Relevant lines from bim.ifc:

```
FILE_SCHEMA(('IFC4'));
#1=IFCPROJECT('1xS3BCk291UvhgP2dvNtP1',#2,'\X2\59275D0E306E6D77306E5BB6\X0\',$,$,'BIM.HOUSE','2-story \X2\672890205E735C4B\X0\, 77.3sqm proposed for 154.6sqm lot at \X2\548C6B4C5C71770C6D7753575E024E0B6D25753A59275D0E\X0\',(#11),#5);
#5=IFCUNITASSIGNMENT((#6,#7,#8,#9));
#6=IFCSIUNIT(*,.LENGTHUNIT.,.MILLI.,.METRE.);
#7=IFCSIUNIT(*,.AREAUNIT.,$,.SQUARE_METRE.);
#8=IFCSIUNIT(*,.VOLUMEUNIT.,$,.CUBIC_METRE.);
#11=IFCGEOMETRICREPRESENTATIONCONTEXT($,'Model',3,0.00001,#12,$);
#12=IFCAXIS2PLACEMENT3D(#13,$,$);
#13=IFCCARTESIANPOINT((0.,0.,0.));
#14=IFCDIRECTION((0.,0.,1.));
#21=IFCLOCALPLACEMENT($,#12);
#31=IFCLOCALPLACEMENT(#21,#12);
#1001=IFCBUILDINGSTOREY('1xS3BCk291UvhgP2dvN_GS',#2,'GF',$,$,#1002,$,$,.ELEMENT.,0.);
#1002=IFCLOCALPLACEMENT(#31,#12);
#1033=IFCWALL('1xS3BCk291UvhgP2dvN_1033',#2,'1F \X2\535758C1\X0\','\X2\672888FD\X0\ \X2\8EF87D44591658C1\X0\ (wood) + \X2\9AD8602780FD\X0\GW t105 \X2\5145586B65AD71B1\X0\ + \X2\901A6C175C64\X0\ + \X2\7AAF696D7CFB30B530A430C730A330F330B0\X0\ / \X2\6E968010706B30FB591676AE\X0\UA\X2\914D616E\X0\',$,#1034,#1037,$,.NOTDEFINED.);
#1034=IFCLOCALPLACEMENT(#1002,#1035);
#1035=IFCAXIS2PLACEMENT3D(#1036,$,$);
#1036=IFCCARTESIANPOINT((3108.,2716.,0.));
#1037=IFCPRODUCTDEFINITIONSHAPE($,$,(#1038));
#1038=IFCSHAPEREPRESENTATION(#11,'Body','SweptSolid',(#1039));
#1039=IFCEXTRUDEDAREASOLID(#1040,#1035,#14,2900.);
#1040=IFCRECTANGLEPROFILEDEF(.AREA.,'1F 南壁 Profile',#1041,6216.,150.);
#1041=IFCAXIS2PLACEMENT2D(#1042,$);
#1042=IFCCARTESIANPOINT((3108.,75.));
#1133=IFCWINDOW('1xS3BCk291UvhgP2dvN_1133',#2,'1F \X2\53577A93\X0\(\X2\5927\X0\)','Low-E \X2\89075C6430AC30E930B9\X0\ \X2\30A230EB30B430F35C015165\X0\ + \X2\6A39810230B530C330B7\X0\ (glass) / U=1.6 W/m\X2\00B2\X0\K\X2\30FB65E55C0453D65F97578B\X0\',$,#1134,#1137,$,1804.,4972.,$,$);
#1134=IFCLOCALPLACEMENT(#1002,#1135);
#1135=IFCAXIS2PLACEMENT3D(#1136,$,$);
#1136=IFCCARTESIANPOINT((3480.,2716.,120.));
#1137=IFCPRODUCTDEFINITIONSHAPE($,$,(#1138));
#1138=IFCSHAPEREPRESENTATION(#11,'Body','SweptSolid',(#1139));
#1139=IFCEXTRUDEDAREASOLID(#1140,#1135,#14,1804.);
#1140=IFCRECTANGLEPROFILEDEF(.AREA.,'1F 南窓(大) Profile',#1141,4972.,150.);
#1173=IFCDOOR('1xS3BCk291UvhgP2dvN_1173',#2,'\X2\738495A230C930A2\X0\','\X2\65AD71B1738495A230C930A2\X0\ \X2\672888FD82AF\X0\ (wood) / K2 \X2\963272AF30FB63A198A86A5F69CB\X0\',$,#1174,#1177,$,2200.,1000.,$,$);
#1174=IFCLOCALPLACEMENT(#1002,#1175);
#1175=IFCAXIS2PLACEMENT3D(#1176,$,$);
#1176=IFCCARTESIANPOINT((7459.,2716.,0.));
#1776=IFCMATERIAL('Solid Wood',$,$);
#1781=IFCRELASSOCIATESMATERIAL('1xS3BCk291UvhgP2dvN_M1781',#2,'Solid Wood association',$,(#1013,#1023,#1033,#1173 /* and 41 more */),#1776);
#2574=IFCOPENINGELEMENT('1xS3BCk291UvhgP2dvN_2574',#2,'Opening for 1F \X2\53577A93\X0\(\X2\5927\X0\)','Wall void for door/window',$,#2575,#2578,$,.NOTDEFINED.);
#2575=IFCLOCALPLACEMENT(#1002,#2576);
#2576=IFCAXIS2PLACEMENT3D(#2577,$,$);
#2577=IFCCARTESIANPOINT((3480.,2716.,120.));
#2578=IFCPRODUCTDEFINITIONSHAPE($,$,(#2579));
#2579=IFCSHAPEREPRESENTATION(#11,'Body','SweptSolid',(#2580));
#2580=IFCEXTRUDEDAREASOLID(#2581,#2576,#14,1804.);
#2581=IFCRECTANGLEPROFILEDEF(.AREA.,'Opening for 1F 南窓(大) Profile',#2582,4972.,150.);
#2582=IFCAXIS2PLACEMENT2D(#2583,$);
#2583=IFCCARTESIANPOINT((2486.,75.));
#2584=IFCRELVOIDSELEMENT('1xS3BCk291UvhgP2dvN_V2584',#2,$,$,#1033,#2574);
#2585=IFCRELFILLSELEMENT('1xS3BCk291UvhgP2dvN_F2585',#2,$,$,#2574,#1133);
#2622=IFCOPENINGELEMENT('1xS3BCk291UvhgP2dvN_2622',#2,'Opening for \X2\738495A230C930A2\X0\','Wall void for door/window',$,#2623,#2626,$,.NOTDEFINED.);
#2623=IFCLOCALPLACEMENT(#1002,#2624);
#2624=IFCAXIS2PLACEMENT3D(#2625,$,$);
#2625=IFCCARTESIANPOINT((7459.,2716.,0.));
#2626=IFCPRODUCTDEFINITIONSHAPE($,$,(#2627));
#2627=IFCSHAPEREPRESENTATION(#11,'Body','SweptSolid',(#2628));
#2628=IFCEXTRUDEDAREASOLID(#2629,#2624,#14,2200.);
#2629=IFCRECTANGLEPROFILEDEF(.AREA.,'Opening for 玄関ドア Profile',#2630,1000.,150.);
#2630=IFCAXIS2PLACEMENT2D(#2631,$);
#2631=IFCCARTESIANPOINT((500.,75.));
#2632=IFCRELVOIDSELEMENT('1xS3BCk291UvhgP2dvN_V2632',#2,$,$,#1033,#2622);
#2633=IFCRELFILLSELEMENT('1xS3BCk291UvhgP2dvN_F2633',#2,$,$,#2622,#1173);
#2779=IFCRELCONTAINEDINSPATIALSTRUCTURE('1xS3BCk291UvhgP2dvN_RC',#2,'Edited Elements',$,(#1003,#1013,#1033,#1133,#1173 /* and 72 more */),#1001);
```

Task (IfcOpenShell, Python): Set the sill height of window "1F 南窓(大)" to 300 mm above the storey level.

```python
import numpy as np
import ifcopenshell
import ifcopenshell.api.geometry
import ifcopenshell.geom
import ifcopenshell.util.element
import ifcopenshell.util.placement
import ifcopenshell.util.shape
import ifcopenshell.util.unit

model = ifcopenshell.open("bim.ifc")
unit_scale = ifcopenshell.util.unit.calculate_unit_scale(model)

window = model.by_guid("1xS3BCk291UvhgP2dvN_1133")
opening = window.FillsVoids[0].RelatingOpeningElement
storey = ifcopenshell.util.element.get_container(window, ifc_class="IfcBuildingStorey")
level = ifcopenshell.util.placement.get_local_placement(storey.ObjectPlacement)[2, 3]

# The opening's origin need not be at the sill, so measure its lowest point.
shape = ifcopenshell.geom.create_shape(ifcopenshell.geom.settings(), opening)
bottom = ifcopenshell.util.shape.get_shape_bottom_elevation(shape, shape.geometry) / unit_scale
dz = level + 0.3 / unit_scale - bottom

shift = np.array([0.0, 0.0, dz])
# The window is not placed relative to its opening, so move both.
for product in (opening, window):
    matrix = ifcopenshell.util.placement.get_local_placement(product.ObjectPlacement)
    matrix[:3, 3] += shift
    ifcopenshell.api.geometry.edit_object_placement(model, product=product, matrix=matrix, is_si=False)

print(f"moved by {dz * unit_scale:+.3f} m")

model.write("bim_updated.ifc")
```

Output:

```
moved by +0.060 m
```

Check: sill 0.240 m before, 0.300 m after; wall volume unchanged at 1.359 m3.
